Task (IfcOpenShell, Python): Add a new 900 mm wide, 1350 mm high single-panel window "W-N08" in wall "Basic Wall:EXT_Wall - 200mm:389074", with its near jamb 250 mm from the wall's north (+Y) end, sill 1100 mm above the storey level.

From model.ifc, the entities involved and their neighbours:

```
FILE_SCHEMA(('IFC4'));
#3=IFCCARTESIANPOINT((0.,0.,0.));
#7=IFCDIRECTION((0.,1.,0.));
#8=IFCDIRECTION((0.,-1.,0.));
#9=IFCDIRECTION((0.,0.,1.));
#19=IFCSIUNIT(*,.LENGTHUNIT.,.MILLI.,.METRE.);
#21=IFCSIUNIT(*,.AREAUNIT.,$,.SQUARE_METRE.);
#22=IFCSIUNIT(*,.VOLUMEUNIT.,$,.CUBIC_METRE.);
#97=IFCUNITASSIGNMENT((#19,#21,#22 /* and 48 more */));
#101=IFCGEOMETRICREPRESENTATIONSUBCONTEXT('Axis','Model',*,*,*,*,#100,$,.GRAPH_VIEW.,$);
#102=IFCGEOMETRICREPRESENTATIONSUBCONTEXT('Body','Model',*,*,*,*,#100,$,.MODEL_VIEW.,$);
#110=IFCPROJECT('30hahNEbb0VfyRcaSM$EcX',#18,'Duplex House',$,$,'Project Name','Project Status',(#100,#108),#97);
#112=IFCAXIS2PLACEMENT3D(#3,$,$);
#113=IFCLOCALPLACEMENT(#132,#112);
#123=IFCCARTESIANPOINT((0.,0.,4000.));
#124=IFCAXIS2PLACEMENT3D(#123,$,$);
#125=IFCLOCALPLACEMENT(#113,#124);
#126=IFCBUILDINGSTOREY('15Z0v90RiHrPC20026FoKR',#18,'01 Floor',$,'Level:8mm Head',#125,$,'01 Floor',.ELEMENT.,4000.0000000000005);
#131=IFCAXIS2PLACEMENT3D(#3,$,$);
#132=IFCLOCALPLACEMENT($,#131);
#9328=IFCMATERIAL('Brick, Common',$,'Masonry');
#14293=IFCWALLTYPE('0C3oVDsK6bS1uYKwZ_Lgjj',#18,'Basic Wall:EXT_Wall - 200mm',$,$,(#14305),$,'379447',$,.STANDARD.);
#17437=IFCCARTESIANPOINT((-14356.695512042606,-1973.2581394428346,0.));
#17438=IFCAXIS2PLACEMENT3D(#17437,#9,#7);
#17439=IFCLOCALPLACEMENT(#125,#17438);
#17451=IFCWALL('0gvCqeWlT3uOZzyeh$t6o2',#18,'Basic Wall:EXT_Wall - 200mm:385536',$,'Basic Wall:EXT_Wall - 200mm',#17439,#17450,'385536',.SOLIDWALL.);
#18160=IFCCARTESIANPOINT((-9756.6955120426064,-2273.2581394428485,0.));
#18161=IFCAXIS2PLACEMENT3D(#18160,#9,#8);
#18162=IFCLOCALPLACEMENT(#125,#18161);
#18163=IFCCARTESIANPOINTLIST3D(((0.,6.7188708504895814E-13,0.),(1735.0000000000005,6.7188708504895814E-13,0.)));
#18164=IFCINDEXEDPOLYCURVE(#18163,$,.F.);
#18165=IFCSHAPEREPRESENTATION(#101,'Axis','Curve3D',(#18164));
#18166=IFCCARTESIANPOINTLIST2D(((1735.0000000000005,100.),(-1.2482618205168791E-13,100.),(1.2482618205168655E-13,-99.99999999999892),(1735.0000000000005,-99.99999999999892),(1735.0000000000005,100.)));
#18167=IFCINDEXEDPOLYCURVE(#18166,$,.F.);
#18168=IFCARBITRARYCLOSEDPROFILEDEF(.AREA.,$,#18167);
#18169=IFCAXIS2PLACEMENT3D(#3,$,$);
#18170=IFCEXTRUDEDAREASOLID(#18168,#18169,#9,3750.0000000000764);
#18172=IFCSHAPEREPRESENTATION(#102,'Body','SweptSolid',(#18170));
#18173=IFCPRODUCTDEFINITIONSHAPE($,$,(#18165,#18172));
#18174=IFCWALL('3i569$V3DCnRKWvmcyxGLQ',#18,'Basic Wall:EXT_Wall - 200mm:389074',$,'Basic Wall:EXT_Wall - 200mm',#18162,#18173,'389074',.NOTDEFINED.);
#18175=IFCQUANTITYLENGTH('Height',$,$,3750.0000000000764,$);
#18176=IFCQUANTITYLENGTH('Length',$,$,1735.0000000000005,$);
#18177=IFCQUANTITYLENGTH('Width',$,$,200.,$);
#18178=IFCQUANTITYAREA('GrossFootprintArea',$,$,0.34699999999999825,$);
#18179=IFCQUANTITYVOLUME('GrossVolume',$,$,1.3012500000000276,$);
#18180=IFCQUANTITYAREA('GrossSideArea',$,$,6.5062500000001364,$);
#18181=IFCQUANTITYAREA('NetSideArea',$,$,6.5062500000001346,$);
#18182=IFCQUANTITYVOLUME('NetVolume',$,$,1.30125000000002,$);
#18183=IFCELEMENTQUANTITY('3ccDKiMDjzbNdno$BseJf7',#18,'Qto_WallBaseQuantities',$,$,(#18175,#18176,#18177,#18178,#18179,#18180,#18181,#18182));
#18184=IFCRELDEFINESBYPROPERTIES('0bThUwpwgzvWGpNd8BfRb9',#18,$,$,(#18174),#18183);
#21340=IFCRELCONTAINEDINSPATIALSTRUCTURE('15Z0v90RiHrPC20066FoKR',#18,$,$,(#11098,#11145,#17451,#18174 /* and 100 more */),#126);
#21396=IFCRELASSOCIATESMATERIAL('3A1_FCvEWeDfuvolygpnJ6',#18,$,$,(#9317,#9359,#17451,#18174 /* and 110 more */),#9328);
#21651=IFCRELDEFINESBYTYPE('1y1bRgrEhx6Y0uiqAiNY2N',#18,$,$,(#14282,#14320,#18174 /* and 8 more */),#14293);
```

```python
import numpy as np
import ifcopenshell
import ifcopenshell.api.feature
import ifcopenshell.api.geometry
import ifcopenshell.api.pset
import ifcopenshell.api.root
import ifcopenshell.api.spatial
import ifcopenshell.geom
import ifcopenshell.util.element
import ifcopenshell.util.placement
import ifcopenshell.util.representation
import ifcopenshell.util.shape
import ifcopenshell.util.unit

model = ifcopenshell.open("model.ifc")
unit_scale = ifcopenshell.util.unit.calculate_unit_scale(model)
area_scale = ifcopenshell.util.unit.calculate_unit_scale(model, "AREAUNIT")
volume_scale = ifcopenshell.util.unit.calculate_unit_scale(model, "VOLUMEUNIT")
settings = ifcopenshell.geom.settings()


def volume(element):
    """Net volume in cubic metres, openings subtracted."""
    shape = ifcopenshell.geom.create_shape(settings, element)
    return ifcopenshell.util.shape.get_volume(shape.geometry)


wall = model.by_guid("3i569$V3DCnRKWvmcyxGLQ")
storey = ifcopenshell.util.element.get_container(wall, ifc_class="IfcBuildingStorey")
context = ifcopenshell.util.representation.get_context(model, "Model", "Body", "MODEL_VIEW")
before = volume(wall)

width, height, from_end, sill = 0.9, 1.35, 0.25, 1.1  # metres

# The wall runs along its own X axis, and the end named is its -X end.
wall_shape = ifcopenshell.geom.create_shape(settings, wall)
x, y, z = ifcopenshell.util.shape.get_vertices(wall_shape.geometry).T
start = x.min() + from_end
face, thickness = float(y.min()), float(y.max() - y.min())
wall_matrix = ifcopenshell.util.placement.get_local_placement(wall.ObjectPlacement)
level = ifcopenshell.util.placement.get_local_placement(storey.ObjectPlacement)[2, 3]


def in_wall(x, y):
    """Placement at x, y metres in the wall's axes, at sill height."""
    matrix = wall_matrix.copy()
    matrix[:, 3] = wall_matrix @ np.array([x / unit_scale, y / unit_scale, 0.0, 1.0])
    matrix[2, 3] = level + sill / unit_scale
    return matrix


# Opening: a box that overshoots both wall faces by 50 mm.
opening = ifcopenshell.api.root.create_entity(model, ifc_class="IfcOpeningElement", predefined_type="OPENING")
box = ifcopenshell.api.geometry.add_wall_representation(
    model, context=context, length=width, height=height, thickness=thickness + 0.1
)
ifcopenshell.api.geometry.assign_representation(model, product=opening, representation=box)
ifcopenshell.api.geometry.edit_object_placement(model, product=opening, matrix=in_wall(start, face - 0.05), is_si=False)
ifcopenshell.api.feature.add_feature(model, feature=opening, element=wall)

window = ifcopenshell.api.root.create_entity(model, ifc_class="IfcWindow", name="W-N08", predefined_type="WINDOW")
window.OverallWidth, window.OverallHeight = width / unit_scale, height / unit_scale
window.PartitioningType = "SINGLE_PANEL"
body = ifcopenshell.api.geometry.add_window_representation(
    model,
    context=context,
    overall_width=window.OverallWidth,
    overall_height=window.OverallHeight,
    partition_type="SINGLE_PANEL",
)
ifcopenshell.api.geometry.assign_representation(model, product=window, representation=body)
ifcopenshell.api.spatial.assign_container(model, products=[window], relating_structure=storey)
ifcopenshell.api.feature.add_filling(model, opening=opening, element=window)

# Centre the window in the wall's thickness.
ifcopenshell.api.geometry.edit_object_placement(model, product=window, matrix=in_wall(start, face), is_si=False)
window_shape = ifcopenshell.geom.create_shape(settings, window)
depth = ifcopenshell.util.shape.get_vertices(window_shape.geometry)[:, 1]
offset = face + thickness / 2 - (depth.min() + depth.max()) / 2
ifcopenshell.api.geometry.edit_object_placement(model, product=window, matrix=in_wall(start, offset), is_si=False)

after = volume(wall)

# Update the wall's stored quantities.
qto = model.by_id(ifcopenshell.util.element.get_pset(wall, "Qto_WallBaseQuantities", should_inherit=False)["id"])
ifcopenshell.api.pset.edit_qto(model, qto=qto, properties={
    "NetSideArea": after / thickness / area_scale,
    "NetVolume": after / volume_scale,
})

print(f"wall volume {before:.3f} -> {after:.3f} m3")

model.write("model_rev.ifc")
```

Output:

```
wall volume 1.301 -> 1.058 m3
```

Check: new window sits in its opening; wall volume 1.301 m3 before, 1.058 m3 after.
